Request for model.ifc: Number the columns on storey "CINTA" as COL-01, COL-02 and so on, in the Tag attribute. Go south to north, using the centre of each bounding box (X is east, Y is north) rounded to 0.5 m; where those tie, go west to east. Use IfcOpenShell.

First a look at what the model holds.

```python
import ifcopenshell
import ifcopenshell.util.element
import ifcopenshell.util.placement

model = ifcopenshell.open("model.ifc")
print(model.schema)
storey = next(s for s in model.by_type("IfcBuildingStorey") if s.Name == "CINTA")
columns = [e for e in ifcopenshell.util.element.get_decomposition(storey) if e.is_a("IfcColumn")]
for e in sorted(columns, key=lambda e: e.id()):
    origin = ifcopenshell.util.placement.get_local_placement(e.ObjectPlacement)[:3, 3]
    print(e.id(), e.Tag, e.Name, origin.round(2) + 0.0, sep=" | ")
```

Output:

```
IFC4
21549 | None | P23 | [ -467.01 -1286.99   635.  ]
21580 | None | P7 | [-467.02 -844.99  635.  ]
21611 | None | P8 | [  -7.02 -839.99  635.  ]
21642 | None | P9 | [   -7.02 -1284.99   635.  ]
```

```python
import ifcopenshell
import ifcopenshell.geom
import ifcopenshell.util.element
import ifcopenshell.util.shape

model = ifcopenshell.open("model.ifc")
settings = ifcopenshell.geom.settings()
settings.set("use-world-coords", True)


def centre(element):
    shape = ifcopenshell.geom.create_shape(settings, element)
    return ifcopenshell.util.shape.get_bbox_centroid(shape.geometry)


storey = next(s for s in model.by_type("IfcBuildingStorey") if s.Name == "CINTA")
columns = [e for e in ifcopenshell.util.element.get_decomposition(storey) if e.is_a("IfcColumn")]

# Insertion points can sit at a corner or the storey origin, so sort by the geometry (in metres).
centres = {e: centre(e) for e in columns}
columns.sort(key=lambda e: (round(centres[e][1] / 0.5), centres[e][0]))

for i, e in enumerate(columns, start=1):
    number = f"COL-{i:02d}"
    e.Tag = number
    print(e.id(), number)

model.write("model_v2.ifc")
```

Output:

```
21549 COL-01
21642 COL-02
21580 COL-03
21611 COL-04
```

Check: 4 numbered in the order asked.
